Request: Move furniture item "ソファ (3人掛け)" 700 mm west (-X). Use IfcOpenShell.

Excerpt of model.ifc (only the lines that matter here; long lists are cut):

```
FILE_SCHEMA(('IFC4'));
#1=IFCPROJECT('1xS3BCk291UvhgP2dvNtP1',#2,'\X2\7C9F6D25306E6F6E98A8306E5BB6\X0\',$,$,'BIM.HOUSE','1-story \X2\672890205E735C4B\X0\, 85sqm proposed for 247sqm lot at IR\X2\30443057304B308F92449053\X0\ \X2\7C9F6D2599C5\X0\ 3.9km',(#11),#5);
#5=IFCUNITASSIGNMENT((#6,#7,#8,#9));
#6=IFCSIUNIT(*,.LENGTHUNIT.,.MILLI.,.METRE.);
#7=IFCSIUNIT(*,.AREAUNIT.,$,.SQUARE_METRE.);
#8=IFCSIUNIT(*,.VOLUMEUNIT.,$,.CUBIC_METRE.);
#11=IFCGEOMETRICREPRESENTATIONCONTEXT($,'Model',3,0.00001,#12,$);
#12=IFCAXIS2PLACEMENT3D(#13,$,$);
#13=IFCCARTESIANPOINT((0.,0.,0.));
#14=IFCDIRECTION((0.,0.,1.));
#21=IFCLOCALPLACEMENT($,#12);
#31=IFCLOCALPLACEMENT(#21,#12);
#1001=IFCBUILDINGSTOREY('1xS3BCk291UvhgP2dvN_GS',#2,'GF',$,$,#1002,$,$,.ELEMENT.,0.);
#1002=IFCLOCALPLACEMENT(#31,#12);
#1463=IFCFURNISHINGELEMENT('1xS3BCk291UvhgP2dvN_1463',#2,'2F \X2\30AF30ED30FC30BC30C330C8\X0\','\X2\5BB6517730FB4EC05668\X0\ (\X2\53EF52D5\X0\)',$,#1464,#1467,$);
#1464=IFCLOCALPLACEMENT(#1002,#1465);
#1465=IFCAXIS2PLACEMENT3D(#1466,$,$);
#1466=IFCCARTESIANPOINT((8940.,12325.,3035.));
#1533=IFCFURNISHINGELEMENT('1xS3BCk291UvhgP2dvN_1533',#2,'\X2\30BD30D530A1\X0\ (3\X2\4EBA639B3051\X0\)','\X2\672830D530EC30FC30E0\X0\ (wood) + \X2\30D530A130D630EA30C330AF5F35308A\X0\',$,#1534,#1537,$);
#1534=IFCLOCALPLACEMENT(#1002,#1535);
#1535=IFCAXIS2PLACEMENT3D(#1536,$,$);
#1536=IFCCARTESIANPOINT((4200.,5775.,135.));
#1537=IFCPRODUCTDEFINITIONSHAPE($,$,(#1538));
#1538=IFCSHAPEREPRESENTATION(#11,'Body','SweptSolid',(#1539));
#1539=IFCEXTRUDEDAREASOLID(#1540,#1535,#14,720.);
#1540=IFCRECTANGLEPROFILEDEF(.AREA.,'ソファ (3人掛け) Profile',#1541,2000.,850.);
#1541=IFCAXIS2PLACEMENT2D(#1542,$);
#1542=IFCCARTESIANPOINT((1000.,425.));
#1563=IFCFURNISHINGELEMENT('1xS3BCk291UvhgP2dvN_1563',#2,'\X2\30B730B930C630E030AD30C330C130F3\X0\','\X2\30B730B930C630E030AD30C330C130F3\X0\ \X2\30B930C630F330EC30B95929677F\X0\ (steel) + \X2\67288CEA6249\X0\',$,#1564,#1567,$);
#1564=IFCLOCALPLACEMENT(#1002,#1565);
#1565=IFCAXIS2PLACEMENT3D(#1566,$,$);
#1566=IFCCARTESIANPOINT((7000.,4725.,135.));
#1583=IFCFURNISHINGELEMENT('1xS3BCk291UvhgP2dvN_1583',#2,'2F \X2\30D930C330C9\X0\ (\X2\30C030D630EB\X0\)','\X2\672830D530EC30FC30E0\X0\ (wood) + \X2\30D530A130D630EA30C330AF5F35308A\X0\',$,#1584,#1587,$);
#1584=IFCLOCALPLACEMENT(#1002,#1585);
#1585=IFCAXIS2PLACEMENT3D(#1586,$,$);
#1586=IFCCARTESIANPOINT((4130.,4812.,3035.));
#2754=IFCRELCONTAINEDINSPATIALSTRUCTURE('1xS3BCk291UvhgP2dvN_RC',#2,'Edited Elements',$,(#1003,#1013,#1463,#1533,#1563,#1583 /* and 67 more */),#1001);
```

```python
import ifcopenshell
import ifcopenshell.api.geometry
import ifcopenshell.util.placement
import ifcopenshell.util.unit

model = ifcopenshell.open("model.ifc")
unit_scale = ifcopenshell.util.unit.calculate_unit_scale(model)

item = model.by_guid("1xS3BCk291UvhgP2dvN_1533")
matrix = ifcopenshell.util.placement.get_local_placement(item.ObjectPlacement)
matrix[0, 3] -= 0.7 / unit_scale
ifcopenshell.api.geometry.edit_object_placement(model, product=item, matrix=matrix, is_si=False)

print(ifcopenshell.util.placement.get_local_placement(item.ObjectPlacement).round(3) + 0.0)

model.write("model_rev.ifc")
```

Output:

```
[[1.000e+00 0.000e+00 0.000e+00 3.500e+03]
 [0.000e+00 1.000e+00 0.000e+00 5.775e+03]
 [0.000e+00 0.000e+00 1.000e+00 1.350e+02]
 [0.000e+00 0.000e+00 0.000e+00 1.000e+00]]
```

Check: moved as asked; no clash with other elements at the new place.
